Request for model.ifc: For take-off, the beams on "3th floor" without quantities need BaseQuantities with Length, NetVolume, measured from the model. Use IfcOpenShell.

First a look at what the model holds.

```python
import ifcopenshell
import ifcopenshell.util.element
import ifcopenshell.util.unit

model = ifcopenshell.open("model.ifc")
print(model.schema)
for unit_type in ("LENGTHUNIT", "AREAUNIT", "VOLUMEUNIT"):
    print(unit_type, ifcopenshell.util.unit.calculate_unit_scale(model, unit_type))
storey = next(s for s in model.by_type("IfcBuildingStorey") if s.Name == "3th floor")
beams = [e for e in ifcopenshell.util.element.get_decomposition(storey) if e.is_a("IfcBeam")]
for e in sorted(beams, key=lambda e: e.id()):
    print(e.id(), e.is_a(), e.Name, list(ifcopenshell.util.element.get_psets(e, qtos_only=True)), sep=" | ")
```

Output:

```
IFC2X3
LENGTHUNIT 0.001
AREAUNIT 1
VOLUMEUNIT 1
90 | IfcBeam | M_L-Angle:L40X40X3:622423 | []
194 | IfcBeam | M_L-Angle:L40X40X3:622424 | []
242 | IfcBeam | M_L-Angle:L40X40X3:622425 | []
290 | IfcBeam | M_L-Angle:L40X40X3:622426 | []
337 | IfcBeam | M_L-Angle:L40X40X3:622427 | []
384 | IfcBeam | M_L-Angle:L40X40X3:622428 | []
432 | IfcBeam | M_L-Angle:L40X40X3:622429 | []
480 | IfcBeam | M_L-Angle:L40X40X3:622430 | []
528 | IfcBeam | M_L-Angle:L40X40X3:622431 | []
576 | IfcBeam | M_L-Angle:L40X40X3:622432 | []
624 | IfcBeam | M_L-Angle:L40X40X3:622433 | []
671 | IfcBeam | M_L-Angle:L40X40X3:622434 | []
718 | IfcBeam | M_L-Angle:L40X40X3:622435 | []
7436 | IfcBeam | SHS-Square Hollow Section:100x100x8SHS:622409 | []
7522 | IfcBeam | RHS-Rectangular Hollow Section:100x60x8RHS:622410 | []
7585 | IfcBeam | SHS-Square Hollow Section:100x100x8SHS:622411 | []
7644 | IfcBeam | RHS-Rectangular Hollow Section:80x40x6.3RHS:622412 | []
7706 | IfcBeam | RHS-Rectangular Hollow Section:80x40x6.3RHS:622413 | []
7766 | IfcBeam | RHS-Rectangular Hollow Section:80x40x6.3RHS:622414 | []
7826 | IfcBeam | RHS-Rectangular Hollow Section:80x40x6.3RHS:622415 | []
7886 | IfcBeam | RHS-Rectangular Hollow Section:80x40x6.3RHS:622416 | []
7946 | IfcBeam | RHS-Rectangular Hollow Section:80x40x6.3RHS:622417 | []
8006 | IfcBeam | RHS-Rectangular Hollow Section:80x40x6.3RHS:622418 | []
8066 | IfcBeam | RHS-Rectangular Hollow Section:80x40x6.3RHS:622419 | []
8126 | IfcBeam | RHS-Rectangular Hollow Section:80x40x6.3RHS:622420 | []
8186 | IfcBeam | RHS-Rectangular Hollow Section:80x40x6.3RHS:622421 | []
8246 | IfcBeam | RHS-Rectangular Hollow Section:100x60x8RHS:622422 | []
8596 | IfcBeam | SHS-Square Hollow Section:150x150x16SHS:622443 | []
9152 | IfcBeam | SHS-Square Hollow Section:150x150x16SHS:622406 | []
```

```python
import ifcopenshell
import ifcopenshell.api.pset
import ifcopenshell.geom
import ifcopenshell.util.element
import ifcopenshell.util.shape
import ifcopenshell.util.unit

model = ifcopenshell.open("model.ifc")
unit_scale = ifcopenshell.util.unit.calculate_unit_scale(model)
volume_scale = ifcopenshell.util.unit.calculate_unit_scale(model, "VOLUMEUNIT")
settings = ifcopenshell.geom.settings()

storey = next(s for s in model.by_type("IfcBuildingStorey") if s.Name == "3th floor")
beams = [e for e in ifcopenshell.util.element.get_decomposition(storey) if e.is_a("IfcBeam")]

for e in sorted(beams, key=lambda e: e.id()):
    if ifcopenshell.util.element.get_psets(e, qtos_only=True, should_inherit=False):
        continue
    # Geometry comes back in metres, in the element's own axes.
    shape = ifcopenshell.geom.create_shape(settings, e)
    values = {
        "Length": ifcopenshell.util.shape.get_max_xyz(shape.geometry) / unit_scale,
        "NetVolume": ifcopenshell.util.shape.get_volume(shape.geometry) / volume_scale,
    }
    qto = ifcopenshell.api.pset.add_qto(model, product=e, name="BaseQuantities")
    ifcopenshell.api.pset.edit_qto(model, qto=qto, properties=values)
    print(e.id(), {k: round(v, 3) for k, v in values.items()})

model.write("model_v2.ifc")
```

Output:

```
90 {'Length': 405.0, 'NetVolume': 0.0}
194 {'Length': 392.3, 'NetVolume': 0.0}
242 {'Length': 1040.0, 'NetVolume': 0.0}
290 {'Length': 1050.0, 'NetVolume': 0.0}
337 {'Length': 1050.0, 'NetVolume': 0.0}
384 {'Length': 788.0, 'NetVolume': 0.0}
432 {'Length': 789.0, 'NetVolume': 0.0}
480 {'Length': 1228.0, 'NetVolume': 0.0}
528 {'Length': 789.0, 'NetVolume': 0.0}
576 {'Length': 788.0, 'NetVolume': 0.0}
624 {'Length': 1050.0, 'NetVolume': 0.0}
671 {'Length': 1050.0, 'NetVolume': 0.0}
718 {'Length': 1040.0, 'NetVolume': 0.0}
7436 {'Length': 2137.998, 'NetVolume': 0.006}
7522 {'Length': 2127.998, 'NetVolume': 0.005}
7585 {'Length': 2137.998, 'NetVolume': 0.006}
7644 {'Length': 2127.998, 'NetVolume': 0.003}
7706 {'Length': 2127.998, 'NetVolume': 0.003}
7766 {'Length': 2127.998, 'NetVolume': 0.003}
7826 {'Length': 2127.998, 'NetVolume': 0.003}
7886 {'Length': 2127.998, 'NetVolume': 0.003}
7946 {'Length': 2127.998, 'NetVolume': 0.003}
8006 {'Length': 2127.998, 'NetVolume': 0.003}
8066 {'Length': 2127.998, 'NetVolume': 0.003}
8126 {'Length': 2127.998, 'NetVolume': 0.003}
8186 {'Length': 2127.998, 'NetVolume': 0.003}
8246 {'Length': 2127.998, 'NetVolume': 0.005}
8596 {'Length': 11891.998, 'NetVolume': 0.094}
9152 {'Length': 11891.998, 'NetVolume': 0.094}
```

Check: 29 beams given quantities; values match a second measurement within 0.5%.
